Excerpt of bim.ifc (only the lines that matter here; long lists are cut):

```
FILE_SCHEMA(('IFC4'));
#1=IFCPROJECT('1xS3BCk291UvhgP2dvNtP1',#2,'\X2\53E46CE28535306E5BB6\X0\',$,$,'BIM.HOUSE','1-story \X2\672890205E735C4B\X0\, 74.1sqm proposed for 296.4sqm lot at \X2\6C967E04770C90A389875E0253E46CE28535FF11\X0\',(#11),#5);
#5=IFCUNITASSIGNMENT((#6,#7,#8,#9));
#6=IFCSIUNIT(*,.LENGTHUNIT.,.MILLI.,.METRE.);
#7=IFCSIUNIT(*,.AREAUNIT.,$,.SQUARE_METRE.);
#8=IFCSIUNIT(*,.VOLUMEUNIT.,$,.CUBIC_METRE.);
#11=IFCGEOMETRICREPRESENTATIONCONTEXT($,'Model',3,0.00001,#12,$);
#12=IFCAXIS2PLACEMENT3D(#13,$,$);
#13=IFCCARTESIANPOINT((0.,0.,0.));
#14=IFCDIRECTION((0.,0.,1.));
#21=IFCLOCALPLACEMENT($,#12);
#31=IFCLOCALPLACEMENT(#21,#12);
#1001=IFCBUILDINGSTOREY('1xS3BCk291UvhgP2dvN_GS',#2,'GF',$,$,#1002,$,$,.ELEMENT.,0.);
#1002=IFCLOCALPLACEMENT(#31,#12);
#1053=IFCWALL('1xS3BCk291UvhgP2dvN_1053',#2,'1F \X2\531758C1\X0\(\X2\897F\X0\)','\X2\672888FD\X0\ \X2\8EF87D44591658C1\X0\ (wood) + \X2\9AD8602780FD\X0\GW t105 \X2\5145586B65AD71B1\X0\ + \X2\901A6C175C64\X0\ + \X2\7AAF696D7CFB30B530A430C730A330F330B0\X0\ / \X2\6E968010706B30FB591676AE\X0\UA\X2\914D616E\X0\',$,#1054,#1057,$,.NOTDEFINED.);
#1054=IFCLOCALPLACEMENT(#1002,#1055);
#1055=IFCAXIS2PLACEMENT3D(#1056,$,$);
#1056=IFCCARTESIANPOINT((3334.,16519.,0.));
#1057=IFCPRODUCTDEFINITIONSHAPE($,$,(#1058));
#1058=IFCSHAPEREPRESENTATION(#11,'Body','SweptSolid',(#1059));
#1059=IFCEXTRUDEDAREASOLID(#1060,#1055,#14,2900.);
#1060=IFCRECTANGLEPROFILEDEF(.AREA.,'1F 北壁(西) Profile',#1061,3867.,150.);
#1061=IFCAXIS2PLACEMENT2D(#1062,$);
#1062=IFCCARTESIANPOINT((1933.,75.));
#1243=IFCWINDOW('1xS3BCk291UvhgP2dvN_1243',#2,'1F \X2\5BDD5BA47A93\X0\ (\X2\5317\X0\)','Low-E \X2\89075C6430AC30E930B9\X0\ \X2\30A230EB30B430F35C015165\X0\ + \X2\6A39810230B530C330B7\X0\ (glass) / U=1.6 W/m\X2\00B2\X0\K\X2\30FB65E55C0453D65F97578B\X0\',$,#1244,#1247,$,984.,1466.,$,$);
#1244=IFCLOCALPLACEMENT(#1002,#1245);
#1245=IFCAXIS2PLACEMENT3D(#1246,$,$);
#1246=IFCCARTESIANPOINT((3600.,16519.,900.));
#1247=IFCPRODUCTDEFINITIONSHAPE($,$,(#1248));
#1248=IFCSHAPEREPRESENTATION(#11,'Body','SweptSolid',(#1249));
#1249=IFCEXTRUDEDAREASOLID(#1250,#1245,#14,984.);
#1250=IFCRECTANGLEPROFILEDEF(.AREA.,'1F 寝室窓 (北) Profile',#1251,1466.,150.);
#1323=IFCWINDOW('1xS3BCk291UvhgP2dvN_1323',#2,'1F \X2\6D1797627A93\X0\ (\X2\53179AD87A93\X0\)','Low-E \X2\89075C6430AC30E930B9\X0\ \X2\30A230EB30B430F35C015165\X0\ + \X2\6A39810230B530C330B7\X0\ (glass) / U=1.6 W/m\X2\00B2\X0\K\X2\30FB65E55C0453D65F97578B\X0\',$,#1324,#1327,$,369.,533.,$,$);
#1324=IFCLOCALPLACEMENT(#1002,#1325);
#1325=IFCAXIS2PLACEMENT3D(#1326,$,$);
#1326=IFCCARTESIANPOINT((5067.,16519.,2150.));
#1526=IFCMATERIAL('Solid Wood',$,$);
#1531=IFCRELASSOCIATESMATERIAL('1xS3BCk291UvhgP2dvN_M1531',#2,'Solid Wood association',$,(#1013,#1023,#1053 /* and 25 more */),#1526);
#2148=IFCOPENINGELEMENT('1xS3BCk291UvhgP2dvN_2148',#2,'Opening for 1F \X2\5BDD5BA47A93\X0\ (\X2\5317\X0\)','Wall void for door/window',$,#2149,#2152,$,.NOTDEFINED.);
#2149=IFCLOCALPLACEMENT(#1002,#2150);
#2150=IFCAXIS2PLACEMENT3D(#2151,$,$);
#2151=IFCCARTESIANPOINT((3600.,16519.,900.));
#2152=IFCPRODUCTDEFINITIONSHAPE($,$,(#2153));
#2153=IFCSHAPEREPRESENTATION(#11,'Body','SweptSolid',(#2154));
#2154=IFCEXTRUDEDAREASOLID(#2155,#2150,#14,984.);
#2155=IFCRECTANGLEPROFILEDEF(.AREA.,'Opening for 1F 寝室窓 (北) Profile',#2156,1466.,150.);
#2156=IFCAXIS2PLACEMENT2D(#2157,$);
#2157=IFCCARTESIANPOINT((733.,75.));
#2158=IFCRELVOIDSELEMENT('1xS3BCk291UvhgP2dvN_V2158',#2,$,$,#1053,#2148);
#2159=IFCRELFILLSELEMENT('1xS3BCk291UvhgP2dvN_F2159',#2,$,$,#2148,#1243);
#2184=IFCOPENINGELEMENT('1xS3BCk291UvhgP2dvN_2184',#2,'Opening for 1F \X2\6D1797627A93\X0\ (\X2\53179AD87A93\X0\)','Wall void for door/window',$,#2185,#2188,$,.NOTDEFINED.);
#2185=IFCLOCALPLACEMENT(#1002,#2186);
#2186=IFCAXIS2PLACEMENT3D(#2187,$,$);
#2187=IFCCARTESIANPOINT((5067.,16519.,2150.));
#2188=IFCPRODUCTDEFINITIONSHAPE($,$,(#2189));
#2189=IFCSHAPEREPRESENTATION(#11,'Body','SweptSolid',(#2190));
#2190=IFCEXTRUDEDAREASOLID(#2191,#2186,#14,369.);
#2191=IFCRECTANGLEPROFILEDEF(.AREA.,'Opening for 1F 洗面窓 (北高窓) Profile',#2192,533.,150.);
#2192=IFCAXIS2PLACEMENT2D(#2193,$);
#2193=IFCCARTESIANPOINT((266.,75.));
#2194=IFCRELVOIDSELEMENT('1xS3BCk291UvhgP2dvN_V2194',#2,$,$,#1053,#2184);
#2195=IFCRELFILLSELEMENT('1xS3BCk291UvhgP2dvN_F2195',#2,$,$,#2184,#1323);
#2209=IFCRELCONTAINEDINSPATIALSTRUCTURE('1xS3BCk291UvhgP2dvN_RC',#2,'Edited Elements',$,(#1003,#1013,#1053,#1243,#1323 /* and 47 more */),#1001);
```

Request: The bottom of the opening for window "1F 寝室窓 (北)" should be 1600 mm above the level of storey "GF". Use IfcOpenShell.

```python
import numpy as np
import ifcopenshell
import ifcopenshell.api.geometry
import ifcopenshell.geom
import ifcopenshell.util.element
import ifcopenshell.util.placement
import ifcopenshell.util.shape
import ifcopenshell.util.unit

model = ifcopenshell.open("bim.ifc")
unit_scale = ifcopenshell.util.unit.calculate_unit_scale(model)

window = model.by_guid("1xS3BCk291UvhgP2dvN_1243")
opening = window.FillsVoids[0].RelatingOpeningElement
storey = ifcopenshell.util.element.get_container(window, ifc_class="IfcBuildingStorey")
level = ifcopenshell.util.placement.get_local_placement(storey.ObjectPlacement)[2, 3]

# The opening's origin need not be at the sill, so measure its lowest point.
shape = ifcopenshell.geom.create_shape(ifcopenshell.geom.settings(), opening)
bottom = ifcopenshell.util.shape.get_shape_bottom_elevation(shape, shape.geometry) / unit_scale
dz = level + 1.6 / unit_scale - bottom

shift = np.array([0.0, 0.0, dz])
# The window is not placed relative to its opening, so move both.
for product in (opening, window):
    matrix = ifcopenshell.util.placement.get_local_placement(product.ObjectPlacement)
    matrix[:3, 3] += shift
    ifcopenshell.api.geometry.edit_object_placement(model, product=product, matrix=matrix, is_si=False)

print(f"moved by {dz * unit_scale:+.3f} m")

model.write("bim_v2.ifc")
```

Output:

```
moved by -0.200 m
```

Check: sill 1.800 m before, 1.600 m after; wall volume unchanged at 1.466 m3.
